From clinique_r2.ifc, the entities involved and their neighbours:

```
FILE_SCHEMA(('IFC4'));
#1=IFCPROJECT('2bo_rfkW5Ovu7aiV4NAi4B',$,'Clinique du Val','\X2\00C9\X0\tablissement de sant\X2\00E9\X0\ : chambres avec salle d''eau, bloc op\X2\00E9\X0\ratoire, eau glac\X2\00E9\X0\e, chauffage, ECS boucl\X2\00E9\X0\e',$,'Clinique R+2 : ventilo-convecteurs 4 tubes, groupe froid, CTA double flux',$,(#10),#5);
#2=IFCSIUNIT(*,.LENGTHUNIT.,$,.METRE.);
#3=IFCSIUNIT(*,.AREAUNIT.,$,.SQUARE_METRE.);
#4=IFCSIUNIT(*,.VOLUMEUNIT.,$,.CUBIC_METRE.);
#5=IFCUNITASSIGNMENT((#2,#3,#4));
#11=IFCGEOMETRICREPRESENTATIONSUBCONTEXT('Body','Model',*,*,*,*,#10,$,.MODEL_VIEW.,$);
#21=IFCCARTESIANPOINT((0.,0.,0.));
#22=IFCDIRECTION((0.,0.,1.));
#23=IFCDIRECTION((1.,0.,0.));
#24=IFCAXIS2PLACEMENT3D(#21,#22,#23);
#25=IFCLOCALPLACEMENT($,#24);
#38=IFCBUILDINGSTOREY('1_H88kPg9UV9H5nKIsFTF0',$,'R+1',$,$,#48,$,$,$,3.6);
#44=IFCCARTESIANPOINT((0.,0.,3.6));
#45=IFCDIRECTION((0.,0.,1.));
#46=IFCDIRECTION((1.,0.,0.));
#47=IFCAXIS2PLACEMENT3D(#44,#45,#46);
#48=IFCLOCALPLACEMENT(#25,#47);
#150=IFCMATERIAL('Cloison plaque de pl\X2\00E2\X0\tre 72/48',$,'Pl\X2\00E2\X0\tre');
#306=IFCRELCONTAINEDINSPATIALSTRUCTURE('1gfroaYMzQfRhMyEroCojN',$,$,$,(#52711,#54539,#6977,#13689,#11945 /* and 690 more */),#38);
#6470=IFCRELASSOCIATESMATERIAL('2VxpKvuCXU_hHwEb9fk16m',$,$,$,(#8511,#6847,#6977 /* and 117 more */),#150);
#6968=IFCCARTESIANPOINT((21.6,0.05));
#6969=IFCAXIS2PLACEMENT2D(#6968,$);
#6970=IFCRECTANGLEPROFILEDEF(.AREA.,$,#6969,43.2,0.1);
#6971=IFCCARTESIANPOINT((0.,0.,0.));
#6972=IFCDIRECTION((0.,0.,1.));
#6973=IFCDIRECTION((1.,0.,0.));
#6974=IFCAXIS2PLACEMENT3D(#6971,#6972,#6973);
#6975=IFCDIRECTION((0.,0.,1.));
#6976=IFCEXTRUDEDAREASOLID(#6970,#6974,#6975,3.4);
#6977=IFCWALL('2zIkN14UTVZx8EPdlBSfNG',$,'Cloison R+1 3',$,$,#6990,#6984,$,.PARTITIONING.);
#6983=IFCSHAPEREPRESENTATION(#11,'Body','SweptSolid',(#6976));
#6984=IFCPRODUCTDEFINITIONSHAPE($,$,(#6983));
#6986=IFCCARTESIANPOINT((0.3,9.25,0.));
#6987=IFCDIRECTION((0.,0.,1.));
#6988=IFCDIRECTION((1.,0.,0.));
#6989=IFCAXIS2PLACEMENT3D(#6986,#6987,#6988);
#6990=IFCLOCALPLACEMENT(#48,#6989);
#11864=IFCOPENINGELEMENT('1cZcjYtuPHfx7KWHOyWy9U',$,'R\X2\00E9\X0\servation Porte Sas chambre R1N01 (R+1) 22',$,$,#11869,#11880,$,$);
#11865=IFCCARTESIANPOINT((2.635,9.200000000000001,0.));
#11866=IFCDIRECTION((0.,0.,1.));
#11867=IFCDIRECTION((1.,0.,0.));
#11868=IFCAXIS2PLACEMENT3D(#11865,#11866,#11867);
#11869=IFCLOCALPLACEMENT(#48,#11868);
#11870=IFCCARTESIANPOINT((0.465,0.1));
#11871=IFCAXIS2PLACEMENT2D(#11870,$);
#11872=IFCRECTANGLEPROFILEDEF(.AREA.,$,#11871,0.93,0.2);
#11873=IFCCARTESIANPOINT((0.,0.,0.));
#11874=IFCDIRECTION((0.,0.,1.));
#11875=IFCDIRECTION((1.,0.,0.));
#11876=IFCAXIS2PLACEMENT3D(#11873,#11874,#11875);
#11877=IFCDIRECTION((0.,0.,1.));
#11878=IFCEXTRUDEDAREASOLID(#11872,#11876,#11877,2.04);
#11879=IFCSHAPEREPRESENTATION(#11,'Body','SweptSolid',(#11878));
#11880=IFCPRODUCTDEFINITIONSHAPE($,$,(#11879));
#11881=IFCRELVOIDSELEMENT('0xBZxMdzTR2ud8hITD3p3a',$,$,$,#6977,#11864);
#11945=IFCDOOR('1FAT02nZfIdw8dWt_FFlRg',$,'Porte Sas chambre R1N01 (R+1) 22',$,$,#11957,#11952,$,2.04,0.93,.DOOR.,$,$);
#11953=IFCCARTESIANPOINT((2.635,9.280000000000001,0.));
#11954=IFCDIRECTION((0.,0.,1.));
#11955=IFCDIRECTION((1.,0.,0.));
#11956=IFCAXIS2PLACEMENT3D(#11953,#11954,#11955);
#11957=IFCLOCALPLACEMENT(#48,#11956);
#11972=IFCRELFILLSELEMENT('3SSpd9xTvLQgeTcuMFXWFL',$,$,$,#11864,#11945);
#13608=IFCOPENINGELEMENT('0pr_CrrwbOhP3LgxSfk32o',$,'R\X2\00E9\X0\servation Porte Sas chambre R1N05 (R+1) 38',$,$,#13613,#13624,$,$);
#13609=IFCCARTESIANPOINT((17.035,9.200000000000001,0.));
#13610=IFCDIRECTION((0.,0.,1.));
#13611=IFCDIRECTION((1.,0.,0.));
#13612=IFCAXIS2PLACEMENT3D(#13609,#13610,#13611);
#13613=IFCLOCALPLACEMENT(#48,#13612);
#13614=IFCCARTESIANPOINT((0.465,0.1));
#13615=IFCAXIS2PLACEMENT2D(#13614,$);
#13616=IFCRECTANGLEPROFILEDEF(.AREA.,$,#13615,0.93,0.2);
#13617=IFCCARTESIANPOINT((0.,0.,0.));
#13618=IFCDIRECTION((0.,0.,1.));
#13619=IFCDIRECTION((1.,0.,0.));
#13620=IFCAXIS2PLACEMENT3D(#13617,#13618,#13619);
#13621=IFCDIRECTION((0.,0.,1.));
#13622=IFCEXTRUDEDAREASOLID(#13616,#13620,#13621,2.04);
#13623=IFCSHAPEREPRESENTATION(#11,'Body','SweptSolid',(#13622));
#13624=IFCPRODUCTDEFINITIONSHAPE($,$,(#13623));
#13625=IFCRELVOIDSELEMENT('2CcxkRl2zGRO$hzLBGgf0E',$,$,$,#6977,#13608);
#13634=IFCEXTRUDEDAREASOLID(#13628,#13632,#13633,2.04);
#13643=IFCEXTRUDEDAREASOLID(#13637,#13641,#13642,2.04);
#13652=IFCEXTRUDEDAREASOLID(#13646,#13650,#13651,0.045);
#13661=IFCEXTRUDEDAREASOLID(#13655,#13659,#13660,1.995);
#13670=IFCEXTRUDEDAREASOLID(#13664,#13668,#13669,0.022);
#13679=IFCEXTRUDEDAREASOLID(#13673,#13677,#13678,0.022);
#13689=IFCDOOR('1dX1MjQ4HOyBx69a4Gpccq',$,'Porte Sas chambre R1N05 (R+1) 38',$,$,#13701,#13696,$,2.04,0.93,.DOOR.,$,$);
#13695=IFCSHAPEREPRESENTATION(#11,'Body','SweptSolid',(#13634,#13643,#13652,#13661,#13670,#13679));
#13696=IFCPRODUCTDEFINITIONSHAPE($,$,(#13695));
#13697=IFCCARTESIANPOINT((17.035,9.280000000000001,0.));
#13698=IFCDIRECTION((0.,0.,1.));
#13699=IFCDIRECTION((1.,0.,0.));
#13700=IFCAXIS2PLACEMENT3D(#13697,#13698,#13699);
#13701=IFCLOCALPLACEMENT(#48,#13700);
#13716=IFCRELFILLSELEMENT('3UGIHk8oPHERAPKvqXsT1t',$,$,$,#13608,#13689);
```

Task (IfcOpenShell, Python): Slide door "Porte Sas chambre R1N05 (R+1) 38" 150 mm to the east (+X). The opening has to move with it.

```python
import ifcopenshell
import ifcopenshell.api.geometry
import ifcopenshell.util.placement
import ifcopenshell.util.unit

model = ifcopenshell.open("clinique_r2.ifc")
unit_scale = ifcopenshell.util.unit.calculate_unit_scale(model)

door = model.by_guid("1dX1MjQ4HOyBx69a4Gpccq")
opening = door.FillsVoids[0].RelatingOpeningElement
wall = opening.VoidsElements[0].RelatingBuildingElement

wall_matrix = ifcopenshell.util.placement.get_local_placement(wall.ObjectPlacement)
shift = wall_matrix[:3, 0] * 0.15 / unit_scale
before = ifcopenshell.util.placement.get_local_placement(door.ObjectPlacement)[:3, 3].copy()

# The door is not placed relative to its opening, so move both.
for product in (opening, door):
    matrix = ifcopenshell.util.placement.get_local_placement(product.ObjectPlacement)
    matrix[:3, 3] += shift
    ifcopenshell.api.geometry.edit_object_placement(model, product=product, matrix=matrix, is_si=False)

after = ifcopenshell.util.placement.get_local_placement(door.ObjectPlacement)[:3, 3]
print("door moved by", (after - before).round(3) + 0.0)

model.write("clinique_r2_v2.ifc")
```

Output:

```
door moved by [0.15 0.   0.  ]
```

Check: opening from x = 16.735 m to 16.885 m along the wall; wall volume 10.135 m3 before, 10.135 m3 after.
